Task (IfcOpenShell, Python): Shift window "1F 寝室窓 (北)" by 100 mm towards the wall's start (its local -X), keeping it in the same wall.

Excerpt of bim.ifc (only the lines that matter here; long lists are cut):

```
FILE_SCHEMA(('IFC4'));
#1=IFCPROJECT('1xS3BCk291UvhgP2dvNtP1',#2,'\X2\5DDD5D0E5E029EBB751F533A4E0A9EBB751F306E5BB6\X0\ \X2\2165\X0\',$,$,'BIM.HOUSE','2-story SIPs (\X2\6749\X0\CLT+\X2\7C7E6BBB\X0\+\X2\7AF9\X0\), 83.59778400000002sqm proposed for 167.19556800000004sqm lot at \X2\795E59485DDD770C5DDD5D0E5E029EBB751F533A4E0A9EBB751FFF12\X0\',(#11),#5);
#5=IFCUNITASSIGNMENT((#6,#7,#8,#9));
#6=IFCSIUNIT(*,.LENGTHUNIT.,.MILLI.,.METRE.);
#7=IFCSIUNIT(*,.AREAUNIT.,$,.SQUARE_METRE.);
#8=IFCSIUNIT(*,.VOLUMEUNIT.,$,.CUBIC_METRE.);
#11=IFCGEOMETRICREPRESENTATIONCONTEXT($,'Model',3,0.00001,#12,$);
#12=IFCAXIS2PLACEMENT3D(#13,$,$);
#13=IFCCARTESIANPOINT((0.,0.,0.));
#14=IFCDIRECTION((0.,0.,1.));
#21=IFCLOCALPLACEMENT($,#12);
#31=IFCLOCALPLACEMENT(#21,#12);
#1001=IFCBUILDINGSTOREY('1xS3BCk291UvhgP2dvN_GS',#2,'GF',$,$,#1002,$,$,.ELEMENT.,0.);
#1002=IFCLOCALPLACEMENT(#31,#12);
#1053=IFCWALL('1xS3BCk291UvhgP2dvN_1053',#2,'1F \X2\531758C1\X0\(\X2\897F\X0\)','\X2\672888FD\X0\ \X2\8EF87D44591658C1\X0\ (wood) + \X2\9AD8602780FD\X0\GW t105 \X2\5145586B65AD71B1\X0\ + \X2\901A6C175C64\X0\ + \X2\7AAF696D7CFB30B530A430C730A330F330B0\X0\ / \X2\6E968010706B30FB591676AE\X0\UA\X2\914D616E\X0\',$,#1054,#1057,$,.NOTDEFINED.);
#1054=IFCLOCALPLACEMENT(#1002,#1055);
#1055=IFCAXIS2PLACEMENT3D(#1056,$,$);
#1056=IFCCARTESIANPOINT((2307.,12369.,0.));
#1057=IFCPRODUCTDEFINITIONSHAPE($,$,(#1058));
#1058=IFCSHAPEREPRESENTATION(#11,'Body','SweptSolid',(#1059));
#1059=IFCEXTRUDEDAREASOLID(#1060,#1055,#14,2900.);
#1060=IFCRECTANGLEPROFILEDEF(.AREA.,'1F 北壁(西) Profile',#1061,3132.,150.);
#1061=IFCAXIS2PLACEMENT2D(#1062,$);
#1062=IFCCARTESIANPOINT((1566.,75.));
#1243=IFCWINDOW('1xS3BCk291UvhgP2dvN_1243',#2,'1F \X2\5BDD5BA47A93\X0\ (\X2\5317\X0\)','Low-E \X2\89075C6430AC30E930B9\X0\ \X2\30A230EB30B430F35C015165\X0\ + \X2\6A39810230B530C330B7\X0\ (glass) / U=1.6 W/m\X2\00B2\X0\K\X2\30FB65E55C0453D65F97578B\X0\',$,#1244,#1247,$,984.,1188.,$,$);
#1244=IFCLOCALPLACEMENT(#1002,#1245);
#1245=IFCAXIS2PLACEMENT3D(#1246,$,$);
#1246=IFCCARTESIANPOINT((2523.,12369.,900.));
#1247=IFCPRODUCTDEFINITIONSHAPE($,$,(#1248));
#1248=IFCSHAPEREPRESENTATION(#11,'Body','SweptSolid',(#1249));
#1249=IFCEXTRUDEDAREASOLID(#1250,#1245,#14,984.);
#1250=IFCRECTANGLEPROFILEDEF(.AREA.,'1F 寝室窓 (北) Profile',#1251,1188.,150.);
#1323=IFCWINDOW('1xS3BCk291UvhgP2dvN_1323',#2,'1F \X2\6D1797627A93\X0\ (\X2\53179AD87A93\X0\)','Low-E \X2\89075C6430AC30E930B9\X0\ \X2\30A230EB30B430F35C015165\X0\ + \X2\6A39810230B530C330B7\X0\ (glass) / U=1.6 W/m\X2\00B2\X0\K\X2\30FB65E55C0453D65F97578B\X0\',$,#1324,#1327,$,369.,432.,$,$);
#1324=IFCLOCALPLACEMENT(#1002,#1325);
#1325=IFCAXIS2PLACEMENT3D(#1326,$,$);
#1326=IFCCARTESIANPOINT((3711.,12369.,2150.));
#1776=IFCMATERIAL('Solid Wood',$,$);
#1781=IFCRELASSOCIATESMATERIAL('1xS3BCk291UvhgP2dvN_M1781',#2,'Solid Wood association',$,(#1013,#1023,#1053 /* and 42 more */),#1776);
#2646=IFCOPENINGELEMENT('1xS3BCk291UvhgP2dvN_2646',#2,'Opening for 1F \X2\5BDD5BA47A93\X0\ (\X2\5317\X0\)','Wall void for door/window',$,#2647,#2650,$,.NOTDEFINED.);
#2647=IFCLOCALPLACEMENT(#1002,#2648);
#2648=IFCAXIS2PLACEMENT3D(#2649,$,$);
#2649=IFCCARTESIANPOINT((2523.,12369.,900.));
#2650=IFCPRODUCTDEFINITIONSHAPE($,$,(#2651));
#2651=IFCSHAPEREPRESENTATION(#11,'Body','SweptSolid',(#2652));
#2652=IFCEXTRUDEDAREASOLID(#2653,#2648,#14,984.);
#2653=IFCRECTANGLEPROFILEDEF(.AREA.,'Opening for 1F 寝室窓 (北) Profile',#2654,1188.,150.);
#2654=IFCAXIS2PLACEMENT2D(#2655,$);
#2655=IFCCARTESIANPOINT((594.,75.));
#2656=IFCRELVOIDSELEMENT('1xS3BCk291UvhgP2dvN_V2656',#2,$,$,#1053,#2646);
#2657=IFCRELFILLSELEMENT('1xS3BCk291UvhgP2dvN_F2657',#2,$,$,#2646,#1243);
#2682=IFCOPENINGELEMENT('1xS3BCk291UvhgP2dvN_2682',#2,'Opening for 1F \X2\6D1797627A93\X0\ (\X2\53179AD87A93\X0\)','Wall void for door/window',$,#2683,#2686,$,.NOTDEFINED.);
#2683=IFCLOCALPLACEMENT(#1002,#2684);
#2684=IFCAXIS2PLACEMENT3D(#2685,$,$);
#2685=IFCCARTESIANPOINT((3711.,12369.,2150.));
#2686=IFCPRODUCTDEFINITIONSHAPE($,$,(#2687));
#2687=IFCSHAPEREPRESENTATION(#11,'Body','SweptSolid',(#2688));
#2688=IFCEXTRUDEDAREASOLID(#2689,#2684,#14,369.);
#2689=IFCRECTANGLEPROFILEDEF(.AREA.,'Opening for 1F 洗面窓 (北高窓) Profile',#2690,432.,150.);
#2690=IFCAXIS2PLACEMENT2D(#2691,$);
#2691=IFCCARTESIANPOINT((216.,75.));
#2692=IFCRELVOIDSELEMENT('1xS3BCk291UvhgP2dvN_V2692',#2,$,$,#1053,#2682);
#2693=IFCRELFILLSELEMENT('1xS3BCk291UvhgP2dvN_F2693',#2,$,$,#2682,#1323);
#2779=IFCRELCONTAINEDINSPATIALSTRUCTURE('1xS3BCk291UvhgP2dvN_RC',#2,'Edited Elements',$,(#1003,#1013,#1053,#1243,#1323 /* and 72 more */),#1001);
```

```python
import ifcopenshell
import ifcopenshell.api.geometry
import ifcopenshell.util.placement
import ifcopenshell.util.unit

model = ifcopenshell.open("bim.ifc")
unit_scale = ifcopenshell.util.unit.calculate_unit_scale(model)

window = model.by_guid("1xS3BCk291UvhgP2dvN_1243")
opening = window.FillsVoids[0].RelatingOpeningElement
wall = opening.VoidsElements[0].RelatingBuildingElement

wall_matrix = ifcopenshell.util.placement.get_local_placement(wall.ObjectPlacement)
shift = wall_matrix[:3, 0] * -0.1 / unit_scale
before = ifcopenshell.util.placement.get_local_placement(window.ObjectPlacement)[:3, 3].copy()

# The window is not placed relative to its opening, so move both.
for product in (opening, window):
    matrix = ifcopenshell.util.placement.get_local_placement(product.ObjectPlacement)
    matrix[:3, 3] += shift
    ifcopenshell.api.geometry.edit_object_placement(model, product=product, matrix=matrix, is_si=False)

after = ifcopenshell.util.placement.get_local_placement(window.ObjectPlacement)[:3, 3]
print("window moved by", (after - before).round(3) + 0.0)

model.write("bim_updated.ifc")
```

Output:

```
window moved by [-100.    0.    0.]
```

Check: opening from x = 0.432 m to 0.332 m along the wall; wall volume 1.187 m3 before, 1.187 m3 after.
